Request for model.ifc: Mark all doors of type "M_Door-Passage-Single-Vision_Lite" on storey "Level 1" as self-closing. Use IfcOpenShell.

First a look at what the model holds.

```python
import ifcopenshell
import ifcopenshell.util.element

model = ifcopenshell.open("model.ifc")
print(model.schema)
storey = next(s for s in model.by_type("IfcBuildingStorey") if s.Name == "Level 1")
doors = [e for e in ifcopenshell.util.element.get_decomposition(storey) if e.is_a("IfcDoor")]
seen = {}
for e in doors:
    element_type = ifcopenshell.util.element.get_type(e)
    key = (element_type.Name if element_type != e and element_type else None, ifcopenshell.util.element.get_pset(e, "Pset_DoorCommon", "SelfClosing"))
    seen[key] = seen.get(key, 0) + 1
for (name, value), count in sorted(seen.items(), key=str):
    print(count, "x", name, "|", value)
```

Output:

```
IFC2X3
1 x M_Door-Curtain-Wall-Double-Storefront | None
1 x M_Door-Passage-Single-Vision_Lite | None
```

```python
import ifcopenshell
import ifcopenshell.api.pset
import ifcopenshell.util.element

model = ifcopenshell.open("model.ifc")

storey = next(s for s in model.by_type("IfcBuildingStorey") if s.Name == "Level 1")
doors = [e for e in ifcopenshell.util.element.get_decomposition(storey) if e.is_a("IfcDoor")]

count = 0
for e in doors:
    element_type = ifcopenshell.util.element.get_type(e)
    if element_type in (None, e) or element_type.Name != "M_Door-Passage-Single-Vision_Lite":
        continue
    # add_pset returns the element's existing set when there is one.
    pset = ifcopenshell.api.pset.add_pset(model, product=e, name="Pset_DoorCommon")
    ifcopenshell.api.pset.edit_pset(model, pset=pset, properties={"SelfClosing": True})
    count += 1

print(count, "doors updated")

model.write("model_edited.ifc")
```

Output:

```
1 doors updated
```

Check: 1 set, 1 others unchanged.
